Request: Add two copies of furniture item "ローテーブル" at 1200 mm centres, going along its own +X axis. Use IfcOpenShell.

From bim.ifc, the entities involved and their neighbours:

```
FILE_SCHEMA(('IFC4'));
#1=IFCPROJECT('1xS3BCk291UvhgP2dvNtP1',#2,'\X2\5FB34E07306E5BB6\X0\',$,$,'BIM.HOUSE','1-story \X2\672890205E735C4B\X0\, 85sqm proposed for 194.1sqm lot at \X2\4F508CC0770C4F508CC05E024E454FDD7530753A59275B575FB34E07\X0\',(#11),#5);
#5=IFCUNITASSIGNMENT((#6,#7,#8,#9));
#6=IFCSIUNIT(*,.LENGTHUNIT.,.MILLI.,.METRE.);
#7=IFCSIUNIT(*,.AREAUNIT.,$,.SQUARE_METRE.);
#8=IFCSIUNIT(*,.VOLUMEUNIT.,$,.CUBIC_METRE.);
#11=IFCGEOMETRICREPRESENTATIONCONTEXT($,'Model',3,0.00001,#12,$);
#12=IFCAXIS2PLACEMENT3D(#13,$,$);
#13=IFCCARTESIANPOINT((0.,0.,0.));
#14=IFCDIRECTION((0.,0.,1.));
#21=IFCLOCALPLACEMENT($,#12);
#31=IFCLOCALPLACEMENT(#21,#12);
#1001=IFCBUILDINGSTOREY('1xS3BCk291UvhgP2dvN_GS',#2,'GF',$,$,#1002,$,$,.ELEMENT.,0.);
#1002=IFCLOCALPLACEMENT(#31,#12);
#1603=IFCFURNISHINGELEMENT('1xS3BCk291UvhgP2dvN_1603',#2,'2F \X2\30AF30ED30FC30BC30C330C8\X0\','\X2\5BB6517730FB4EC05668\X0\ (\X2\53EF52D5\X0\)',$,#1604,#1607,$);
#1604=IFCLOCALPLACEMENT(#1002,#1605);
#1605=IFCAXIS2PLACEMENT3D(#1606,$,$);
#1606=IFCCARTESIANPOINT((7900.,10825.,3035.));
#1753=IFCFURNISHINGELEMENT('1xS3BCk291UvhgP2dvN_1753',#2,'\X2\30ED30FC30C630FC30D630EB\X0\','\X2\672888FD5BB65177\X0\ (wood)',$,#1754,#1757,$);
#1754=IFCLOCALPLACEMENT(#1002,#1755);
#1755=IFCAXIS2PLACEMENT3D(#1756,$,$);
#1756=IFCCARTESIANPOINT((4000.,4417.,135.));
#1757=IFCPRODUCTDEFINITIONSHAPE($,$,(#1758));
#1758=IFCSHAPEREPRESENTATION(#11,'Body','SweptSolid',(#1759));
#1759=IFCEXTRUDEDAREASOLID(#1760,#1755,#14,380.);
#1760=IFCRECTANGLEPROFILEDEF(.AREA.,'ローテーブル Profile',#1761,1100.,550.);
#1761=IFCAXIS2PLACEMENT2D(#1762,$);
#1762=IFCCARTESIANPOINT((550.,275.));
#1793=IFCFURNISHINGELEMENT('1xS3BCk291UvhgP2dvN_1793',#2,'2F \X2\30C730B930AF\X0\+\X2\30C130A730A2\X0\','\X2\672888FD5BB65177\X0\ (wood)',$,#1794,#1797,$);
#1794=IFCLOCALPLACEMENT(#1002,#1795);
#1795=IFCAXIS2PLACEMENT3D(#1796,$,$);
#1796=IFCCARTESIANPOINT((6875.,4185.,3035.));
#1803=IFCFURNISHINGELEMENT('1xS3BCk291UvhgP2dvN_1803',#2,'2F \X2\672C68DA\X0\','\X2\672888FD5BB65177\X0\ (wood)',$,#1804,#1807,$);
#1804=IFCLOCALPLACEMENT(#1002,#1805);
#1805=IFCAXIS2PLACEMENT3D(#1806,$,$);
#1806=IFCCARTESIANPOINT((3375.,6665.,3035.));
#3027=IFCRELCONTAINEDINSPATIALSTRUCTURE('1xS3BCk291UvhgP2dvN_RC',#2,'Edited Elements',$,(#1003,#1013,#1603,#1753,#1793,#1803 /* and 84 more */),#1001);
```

```python
import ifcopenshell
import ifcopenshell.api.geometry
import ifcopenshell.api.root
import ifcopenshell.util.element
import ifcopenshell.util.placement

model = ifcopenshell.open("bim.ifc")


def reuse_history(source, copy):
    """copy_class also copies each property set's owner history, people and application; keep the originals."""
    for rel in copy.IsDefinedBy:
        if rel.is_a("IfcRelDefinesByProperties") and (history := rel.RelatingPropertyDefinition.OwnerHistory):
            rel.RelatingPropertyDefinition.OwnerHistory = source.OwnerHistory
            ifcopenshell.util.element.remove_deep2(model, history)


source = model.by_id(1753)
base = ifcopenshell.util.placement.get_local_placement(source.ObjectPlacement)
step = base[:3, 0] * 1200.0

for i in range(1, 3):
    copy = ifcopenshell.api.root.copy_class(model, product=source)
    copy.Representation = ifcopenshell.util.element.copy_deep(
        model, source.Representation, exclude=["IfcGeometricRepresentationContext", "IfcRepresentationMap"]
    )
    reuse_history(source, copy)
    matrix = base.copy()
    matrix[:3, 3] += i * step
    print("added at", matrix[:3, 3].round(3) + 0.0)
    ifcopenshell.api.geometry.edit_object_placement(model, product=copy, matrix=matrix, is_si=False)

model.write("bim_updated.ifc")
```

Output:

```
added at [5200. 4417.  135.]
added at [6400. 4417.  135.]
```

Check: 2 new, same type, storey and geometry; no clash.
